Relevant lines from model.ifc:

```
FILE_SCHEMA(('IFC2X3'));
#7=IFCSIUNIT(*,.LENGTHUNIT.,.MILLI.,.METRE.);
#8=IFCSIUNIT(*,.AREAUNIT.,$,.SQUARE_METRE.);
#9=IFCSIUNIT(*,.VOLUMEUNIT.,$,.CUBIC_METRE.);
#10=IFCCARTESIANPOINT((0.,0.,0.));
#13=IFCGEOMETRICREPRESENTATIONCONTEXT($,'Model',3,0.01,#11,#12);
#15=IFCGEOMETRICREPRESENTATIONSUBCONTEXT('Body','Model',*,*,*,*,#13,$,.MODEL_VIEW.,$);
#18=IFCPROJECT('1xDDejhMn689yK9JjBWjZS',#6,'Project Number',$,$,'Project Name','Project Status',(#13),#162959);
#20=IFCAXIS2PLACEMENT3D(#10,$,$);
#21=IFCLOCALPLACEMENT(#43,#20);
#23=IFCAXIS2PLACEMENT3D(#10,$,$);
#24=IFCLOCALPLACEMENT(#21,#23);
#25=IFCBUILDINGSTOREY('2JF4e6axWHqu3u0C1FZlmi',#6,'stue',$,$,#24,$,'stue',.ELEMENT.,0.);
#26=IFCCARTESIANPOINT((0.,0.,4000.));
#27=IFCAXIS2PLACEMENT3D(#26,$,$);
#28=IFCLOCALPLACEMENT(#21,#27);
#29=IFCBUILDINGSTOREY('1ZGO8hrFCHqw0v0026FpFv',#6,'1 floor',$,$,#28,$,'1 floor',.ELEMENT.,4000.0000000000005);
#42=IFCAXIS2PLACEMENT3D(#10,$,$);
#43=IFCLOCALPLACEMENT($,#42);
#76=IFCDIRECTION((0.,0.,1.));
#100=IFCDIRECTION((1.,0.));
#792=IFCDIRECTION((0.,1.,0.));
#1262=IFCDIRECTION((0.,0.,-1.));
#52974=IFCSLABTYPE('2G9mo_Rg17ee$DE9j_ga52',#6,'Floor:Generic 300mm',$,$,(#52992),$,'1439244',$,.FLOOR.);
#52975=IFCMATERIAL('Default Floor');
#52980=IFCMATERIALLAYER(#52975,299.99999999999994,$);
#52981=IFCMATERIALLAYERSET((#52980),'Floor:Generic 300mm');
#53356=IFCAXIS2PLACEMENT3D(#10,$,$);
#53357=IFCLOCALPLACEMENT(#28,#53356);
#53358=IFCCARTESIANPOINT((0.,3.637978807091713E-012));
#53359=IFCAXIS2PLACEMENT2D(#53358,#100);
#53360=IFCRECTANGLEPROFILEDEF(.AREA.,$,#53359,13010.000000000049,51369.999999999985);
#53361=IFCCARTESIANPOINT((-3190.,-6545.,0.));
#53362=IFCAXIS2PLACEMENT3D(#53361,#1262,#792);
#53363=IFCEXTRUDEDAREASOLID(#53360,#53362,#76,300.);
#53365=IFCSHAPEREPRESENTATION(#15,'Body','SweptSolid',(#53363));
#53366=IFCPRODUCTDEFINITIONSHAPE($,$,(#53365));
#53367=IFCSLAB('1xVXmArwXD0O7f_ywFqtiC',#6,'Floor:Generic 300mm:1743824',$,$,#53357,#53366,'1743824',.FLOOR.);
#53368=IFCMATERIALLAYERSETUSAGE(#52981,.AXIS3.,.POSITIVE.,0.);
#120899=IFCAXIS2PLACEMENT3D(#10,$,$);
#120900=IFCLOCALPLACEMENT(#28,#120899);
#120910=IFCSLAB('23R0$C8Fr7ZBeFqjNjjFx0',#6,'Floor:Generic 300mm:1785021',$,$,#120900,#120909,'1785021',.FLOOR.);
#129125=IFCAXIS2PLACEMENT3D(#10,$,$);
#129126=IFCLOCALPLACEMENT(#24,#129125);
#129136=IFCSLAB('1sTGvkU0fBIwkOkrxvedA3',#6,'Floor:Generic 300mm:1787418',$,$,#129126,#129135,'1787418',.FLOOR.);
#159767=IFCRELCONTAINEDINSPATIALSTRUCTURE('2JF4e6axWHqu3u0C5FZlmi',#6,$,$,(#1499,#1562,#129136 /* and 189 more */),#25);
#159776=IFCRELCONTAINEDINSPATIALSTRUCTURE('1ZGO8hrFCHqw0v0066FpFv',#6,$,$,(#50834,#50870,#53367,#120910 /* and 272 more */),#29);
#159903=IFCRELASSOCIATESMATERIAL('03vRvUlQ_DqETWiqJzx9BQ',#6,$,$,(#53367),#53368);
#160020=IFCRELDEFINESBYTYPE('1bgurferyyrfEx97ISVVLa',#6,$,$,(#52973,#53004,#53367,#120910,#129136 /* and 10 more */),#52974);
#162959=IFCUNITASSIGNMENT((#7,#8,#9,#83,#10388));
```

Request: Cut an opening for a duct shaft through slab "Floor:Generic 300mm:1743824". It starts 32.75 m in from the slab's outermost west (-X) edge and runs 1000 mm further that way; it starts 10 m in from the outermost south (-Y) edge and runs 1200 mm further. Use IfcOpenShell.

```python
import numpy as np
import ifcopenshell
import ifcopenshell.api.feature
import ifcopenshell.api.geometry
import ifcopenshell.api.root
import ifcopenshell.geom
import ifcopenshell.util.placement
import ifcopenshell.util.representation
import ifcopenshell.util.shape
import ifcopenshell.util.unit

model = ifcopenshell.open("model.ifc")
unit_scale = ifcopenshell.util.unit.calculate_unit_scale(model)
settings = ifcopenshell.geom.settings()


def volume(element):
    """Net volume in cubic metres, openings subtracted."""
    shape = ifcopenshell.geom.create_shape(settings, element)
    return ifcopenshell.util.shape.get_volume(shape.geometry)


slab = model.by_guid("1xVXmArwXD0O7f_ywFqtiC")
before = volume(slab)

# Extent in the slab's own axes, in metres. The edges named are its -X and -Y sides.
slab_shape = ifcopenshell.geom.create_shape(settings, slab)
vertices = ifcopenshell.util.shape.get_vertices(slab_shape.geometry)
x_min, y_min, bottom = vertices.min(axis=0)
top = vertices[:, 2].max()

opening = ifcopenshell.api.root.create_entity(model, ifc_class="IfcOpeningElement", name="Duct shaft opening")
context = ifcopenshell.util.representation.get_context(model, "Model", "Body", "MODEL_VIEW")
width, depth = 1, 1.2
outline = [(0.0, 0.0), (width, 0.0), (width, depth), (0.0, depth), (0.0, 0.0)]
# Overshoot both faces by 50 mm so the cut is clean.
shape = ifcopenshell.api.geometry.add_slab_representation(
    model, context=context, depth=top - bottom + 0.1, polyline=outline
)
ifcopenshell.api.geometry.assign_representation(model, product=opening, representation=shape)

matrix = ifcopenshell.util.placement.get_local_placement(slab.ObjectPlacement)
matrix[:, 3] = matrix @ np.append(np.array([x_min + 32.75, y_min + 10, bottom - 0.05]) / unit_scale, 1.0)
ifcopenshell.api.geometry.edit_object_placement(model, product=opening, matrix=matrix, is_si=False)
ifcopenshell.api.feature.add_feature(model, feature=opening, element=slab)

after = volume(slab)

print(f"slab volume {before:.3f} -> {after:.3f} m3")

model.write("model-out.ifc")
```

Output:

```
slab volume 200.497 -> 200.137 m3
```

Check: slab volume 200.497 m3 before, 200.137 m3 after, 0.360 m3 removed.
